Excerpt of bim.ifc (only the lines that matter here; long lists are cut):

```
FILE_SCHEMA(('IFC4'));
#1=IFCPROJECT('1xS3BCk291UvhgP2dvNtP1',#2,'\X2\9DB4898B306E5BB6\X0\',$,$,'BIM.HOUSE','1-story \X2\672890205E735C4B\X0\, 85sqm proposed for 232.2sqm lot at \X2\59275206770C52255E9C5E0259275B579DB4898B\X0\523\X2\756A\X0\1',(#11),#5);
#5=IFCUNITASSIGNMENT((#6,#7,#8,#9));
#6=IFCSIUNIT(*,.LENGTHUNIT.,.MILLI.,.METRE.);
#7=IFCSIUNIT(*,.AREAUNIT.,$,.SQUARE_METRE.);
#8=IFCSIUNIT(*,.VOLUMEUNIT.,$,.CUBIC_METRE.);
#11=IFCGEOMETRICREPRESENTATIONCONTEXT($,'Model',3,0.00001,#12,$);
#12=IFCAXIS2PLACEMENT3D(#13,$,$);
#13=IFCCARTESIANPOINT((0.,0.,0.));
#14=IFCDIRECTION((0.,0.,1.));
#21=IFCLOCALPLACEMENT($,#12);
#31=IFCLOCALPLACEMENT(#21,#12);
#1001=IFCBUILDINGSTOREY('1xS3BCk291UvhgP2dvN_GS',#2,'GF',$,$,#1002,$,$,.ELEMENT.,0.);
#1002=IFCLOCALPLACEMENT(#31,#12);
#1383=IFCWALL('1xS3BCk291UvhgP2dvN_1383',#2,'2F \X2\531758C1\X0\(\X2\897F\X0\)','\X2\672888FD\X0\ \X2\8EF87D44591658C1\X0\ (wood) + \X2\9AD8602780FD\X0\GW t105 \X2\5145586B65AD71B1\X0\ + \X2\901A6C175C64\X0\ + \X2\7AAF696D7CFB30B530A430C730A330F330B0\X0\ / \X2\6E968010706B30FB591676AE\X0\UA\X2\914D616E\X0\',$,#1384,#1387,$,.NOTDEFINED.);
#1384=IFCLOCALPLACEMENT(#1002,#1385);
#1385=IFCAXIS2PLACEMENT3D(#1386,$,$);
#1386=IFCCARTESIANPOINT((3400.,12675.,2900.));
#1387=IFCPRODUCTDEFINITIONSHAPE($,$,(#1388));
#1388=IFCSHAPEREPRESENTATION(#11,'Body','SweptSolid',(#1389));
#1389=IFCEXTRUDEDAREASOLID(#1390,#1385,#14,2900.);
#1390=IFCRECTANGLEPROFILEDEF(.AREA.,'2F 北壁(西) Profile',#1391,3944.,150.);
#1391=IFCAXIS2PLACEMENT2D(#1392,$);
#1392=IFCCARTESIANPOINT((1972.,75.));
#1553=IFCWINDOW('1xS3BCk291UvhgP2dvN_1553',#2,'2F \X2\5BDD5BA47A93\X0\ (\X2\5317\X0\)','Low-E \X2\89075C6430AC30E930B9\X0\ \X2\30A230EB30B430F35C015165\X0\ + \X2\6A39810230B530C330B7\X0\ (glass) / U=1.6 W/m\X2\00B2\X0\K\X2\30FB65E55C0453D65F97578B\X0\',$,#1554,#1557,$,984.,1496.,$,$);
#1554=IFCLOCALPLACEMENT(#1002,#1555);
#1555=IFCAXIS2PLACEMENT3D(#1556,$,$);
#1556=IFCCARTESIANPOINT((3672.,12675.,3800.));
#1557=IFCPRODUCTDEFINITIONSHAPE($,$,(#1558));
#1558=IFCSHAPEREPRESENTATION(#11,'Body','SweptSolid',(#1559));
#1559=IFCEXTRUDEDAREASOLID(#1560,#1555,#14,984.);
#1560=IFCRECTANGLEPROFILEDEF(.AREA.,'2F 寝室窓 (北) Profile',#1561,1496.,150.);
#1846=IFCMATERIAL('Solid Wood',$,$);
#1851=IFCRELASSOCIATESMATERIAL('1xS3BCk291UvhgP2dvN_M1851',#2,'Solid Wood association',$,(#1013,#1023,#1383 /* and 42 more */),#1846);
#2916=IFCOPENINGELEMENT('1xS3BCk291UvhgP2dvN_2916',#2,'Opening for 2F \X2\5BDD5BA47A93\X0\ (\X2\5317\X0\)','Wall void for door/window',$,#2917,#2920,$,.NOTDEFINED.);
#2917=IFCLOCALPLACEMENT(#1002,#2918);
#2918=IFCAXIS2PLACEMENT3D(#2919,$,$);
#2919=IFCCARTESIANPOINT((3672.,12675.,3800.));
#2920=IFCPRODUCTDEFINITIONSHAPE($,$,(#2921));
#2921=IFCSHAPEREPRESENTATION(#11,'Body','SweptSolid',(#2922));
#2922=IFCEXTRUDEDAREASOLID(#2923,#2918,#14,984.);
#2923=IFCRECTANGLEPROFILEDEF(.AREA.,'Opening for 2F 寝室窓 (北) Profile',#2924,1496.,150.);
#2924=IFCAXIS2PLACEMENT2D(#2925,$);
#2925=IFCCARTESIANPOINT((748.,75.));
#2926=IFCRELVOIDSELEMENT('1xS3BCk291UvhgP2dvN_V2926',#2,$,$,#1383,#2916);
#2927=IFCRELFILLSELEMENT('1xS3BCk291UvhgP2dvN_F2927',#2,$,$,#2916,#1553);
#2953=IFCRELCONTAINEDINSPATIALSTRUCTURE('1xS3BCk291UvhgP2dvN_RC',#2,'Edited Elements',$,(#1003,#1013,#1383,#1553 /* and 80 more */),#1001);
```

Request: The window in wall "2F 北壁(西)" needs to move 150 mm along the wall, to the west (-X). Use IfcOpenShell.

```python
import ifcopenshell
import ifcopenshell.api.geometry
import ifcopenshell.util.placement
import ifcopenshell.util.unit

model = ifcopenshell.open("bim.ifc")
unit_scale = ifcopenshell.util.unit.calculate_unit_scale(model)

window = model.by_id(1553)
opening = window.FillsVoids[0].RelatingOpeningElement
wall = opening.VoidsElements[0].RelatingBuildingElement

wall_matrix = ifcopenshell.util.placement.get_local_placement(wall.ObjectPlacement)
shift = wall_matrix[:3, 0] * -0.15 / unit_scale
before = ifcopenshell.util.placement.get_local_placement(window.ObjectPlacement)[:3, 3].copy()

# The window is not placed relative to its opening, so move both.
for product in (opening, window):
    matrix = ifcopenshell.util.placement.get_local_placement(product.ObjectPlacement)
    matrix[:3, 3] += shift
    ifcopenshell.api.geometry.edit_object_placement(model, product=product, matrix=matrix, is_si=False)

after = ifcopenshell.util.placement.get_local_placement(window.ObjectPlacement)[:3, 3]
print("window moved by", (after - before).round(3) + 0.0)

model.write("bim_updated.ifc")
```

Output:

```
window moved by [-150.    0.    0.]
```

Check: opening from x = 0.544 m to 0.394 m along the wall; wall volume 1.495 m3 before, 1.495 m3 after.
